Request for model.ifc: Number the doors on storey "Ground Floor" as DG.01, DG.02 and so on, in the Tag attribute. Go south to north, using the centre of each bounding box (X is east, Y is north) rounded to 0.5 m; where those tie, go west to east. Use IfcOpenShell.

First a look at what the model holds.

```python
import ifcopenshell
import ifcopenshell.util.element
import ifcopenshell.util.placement

model = ifcopenshell.open("model.ifc")
print(model.schema)
storey = next(s for s in model.by_type("IfcBuildingStorey") if s.Name == "Ground Floor")
doors = [e for e in ifcopenshell.util.element.get_decomposition(storey) if e.is_a("IfcDoor")]
for e in sorted(doors, key=lambda e: e.id()):
    origin = ifcopenshell.util.placement.get_local_placement(e.ObjectPlacement)[:3, 3]
    print(e.id(), e.Tag, e.Name, origin.round(2) + 0.0, sep=" | ")
```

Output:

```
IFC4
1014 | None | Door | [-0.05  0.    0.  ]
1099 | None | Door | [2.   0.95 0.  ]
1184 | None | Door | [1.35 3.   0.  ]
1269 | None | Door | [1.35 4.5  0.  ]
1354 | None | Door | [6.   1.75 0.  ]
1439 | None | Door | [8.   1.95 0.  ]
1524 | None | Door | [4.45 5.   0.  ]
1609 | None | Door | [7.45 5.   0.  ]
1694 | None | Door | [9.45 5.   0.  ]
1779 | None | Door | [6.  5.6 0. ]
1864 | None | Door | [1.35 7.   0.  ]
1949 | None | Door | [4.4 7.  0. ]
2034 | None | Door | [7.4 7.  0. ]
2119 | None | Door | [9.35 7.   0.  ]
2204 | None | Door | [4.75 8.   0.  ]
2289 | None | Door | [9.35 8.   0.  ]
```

```python
import ifcopenshell
import ifcopenshell.geom
import ifcopenshell.util.element
import ifcopenshell.util.shape

model = ifcopenshell.open("model.ifc")
settings = ifcopenshell.geom.settings()
settings.set("use-world-coords", True)


def centre(element):
    shape = ifcopenshell.geom.create_shape(settings, element)
    return ifcopenshell.util.shape.get_bbox_centroid(shape.geometry)


storey = next(s for s in model.by_type("IfcBuildingStorey") if s.Name == "Ground Floor")
doors = [e for e in ifcopenshell.util.element.get_decomposition(storey) if e.is_a("IfcDoor")]

# Insertion points can sit at a corner or the storey origin, so sort by the geometry (in metres).
centres = {e: centre(e) for e in doors}
doors.sort(key=lambda e: (round(centres[e][1] / 0.5), centres[e][0]))

for i, e in enumerate(doors, start=1):
    number = f"DG.{i:02d}"
    e.Tag = number
    print(e.id(), number)

model.write("model_edited.ifc")
```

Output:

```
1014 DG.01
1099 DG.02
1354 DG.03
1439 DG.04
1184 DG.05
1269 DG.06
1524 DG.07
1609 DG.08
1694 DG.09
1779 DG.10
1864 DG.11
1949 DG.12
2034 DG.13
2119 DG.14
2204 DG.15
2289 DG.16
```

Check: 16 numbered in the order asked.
